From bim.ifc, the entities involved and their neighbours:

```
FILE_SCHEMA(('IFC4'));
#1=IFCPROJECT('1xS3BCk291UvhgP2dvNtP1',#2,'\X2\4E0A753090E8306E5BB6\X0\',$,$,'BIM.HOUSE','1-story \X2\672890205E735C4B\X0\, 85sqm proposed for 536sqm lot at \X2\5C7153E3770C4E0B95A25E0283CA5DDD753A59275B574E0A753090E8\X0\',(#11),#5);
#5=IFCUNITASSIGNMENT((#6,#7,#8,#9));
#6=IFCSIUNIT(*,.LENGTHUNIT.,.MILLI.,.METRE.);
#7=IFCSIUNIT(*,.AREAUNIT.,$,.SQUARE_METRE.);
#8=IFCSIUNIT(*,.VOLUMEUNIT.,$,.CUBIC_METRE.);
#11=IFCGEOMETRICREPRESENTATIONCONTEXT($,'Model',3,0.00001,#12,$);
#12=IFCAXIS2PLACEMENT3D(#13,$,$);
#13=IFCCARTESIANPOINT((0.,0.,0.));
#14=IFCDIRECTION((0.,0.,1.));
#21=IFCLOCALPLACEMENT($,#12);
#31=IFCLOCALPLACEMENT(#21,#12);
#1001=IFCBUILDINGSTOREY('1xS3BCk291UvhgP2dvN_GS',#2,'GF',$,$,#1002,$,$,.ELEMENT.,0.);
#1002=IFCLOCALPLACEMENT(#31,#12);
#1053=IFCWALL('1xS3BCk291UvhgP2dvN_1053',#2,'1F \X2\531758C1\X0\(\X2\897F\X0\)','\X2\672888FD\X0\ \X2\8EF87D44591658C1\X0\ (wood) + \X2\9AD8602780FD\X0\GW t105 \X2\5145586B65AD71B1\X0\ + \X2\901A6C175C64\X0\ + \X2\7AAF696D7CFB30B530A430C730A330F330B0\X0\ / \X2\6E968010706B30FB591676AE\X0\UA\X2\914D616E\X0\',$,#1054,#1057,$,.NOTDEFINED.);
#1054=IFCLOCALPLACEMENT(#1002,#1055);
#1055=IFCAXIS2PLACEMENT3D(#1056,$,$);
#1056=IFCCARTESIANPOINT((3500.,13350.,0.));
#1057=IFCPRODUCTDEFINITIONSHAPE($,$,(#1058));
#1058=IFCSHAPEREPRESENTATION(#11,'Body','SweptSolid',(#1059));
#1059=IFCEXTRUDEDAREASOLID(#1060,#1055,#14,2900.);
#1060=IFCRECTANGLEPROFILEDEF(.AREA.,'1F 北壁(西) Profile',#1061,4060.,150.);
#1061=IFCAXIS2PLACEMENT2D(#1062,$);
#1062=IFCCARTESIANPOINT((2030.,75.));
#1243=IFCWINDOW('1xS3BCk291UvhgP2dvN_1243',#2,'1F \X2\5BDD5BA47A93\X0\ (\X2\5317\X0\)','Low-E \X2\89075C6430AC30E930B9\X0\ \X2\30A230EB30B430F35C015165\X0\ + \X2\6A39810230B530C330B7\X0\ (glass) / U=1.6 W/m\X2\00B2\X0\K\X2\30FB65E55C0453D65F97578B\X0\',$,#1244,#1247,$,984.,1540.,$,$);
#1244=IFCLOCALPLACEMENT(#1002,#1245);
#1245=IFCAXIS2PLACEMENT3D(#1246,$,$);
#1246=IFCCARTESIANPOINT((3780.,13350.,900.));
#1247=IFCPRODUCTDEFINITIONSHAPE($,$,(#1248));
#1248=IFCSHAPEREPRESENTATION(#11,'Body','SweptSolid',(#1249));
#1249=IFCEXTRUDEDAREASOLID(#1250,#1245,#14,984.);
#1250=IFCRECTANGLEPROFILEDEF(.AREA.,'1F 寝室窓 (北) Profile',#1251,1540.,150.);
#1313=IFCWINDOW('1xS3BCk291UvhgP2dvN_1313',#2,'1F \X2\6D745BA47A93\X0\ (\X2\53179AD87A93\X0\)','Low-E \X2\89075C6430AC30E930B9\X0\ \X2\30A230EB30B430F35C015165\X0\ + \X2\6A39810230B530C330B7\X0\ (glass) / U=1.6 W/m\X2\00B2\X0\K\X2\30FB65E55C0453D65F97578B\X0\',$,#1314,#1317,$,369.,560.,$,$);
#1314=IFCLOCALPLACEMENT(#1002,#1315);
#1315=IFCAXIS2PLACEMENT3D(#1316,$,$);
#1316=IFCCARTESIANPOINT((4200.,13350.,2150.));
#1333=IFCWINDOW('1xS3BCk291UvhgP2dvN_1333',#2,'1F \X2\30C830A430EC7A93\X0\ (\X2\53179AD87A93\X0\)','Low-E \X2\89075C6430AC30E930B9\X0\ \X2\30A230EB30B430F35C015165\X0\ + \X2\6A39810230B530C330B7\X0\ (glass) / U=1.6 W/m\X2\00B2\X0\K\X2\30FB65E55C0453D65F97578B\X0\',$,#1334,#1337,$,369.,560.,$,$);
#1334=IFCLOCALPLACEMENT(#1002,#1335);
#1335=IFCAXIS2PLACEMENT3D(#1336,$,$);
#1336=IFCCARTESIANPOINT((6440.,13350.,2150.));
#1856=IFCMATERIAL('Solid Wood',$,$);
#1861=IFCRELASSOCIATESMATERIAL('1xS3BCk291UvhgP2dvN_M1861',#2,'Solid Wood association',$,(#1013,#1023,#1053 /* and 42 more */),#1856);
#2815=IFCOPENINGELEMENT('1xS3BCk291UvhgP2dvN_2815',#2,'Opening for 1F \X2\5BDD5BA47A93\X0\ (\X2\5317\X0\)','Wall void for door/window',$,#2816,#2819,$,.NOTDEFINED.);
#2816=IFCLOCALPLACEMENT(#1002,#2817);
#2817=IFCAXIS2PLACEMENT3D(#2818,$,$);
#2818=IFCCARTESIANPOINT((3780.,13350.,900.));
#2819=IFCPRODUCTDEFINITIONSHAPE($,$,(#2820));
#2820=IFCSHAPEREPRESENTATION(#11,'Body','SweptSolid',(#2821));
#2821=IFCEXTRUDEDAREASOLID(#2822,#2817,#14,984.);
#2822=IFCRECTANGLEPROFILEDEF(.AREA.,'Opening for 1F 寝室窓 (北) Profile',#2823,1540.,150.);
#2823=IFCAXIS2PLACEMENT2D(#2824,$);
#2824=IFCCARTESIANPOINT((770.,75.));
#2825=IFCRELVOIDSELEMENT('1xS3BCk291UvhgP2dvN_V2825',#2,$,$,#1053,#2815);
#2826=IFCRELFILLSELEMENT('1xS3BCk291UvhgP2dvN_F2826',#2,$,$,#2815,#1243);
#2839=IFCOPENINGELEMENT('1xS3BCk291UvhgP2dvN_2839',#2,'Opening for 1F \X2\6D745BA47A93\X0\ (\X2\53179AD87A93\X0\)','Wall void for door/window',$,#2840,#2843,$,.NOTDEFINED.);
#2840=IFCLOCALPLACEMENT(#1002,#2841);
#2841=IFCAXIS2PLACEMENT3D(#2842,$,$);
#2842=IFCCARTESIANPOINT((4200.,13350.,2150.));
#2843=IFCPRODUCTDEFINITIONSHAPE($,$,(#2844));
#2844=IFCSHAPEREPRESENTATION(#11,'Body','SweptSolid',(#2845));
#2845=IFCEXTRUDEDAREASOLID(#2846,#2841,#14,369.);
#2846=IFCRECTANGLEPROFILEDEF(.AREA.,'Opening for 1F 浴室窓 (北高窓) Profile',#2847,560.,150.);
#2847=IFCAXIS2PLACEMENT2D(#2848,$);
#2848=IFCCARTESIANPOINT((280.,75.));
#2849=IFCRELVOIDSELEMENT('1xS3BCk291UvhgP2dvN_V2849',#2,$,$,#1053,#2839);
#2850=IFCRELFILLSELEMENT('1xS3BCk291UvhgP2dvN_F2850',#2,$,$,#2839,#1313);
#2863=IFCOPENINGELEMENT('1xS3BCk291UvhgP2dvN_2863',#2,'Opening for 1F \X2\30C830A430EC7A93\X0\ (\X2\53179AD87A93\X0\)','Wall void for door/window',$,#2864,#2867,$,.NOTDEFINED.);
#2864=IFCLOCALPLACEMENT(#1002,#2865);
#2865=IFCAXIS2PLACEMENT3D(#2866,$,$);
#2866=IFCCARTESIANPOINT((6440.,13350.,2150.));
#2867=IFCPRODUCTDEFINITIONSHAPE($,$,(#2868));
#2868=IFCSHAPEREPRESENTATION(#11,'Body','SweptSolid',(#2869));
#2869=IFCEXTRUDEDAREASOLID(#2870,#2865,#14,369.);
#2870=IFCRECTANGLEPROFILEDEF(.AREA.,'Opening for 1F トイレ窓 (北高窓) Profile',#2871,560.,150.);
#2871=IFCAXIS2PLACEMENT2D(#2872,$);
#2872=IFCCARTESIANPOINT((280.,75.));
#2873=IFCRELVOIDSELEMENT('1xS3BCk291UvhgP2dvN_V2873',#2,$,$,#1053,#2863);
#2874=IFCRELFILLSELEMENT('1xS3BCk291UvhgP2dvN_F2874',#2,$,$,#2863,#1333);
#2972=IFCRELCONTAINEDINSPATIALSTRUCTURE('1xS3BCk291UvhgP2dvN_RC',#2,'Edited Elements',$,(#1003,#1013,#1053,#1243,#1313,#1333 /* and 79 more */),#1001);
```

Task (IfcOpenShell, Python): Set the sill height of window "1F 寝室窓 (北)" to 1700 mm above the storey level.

```python
import numpy as np
import ifcopenshell
import ifcopenshell.api.geometry
import ifcopenshell.geom
import ifcopenshell.util.element
import ifcopenshell.util.placement
import ifcopenshell.util.shape
import ifcopenshell.util.unit

model = ifcopenshell.open("bim.ifc")
unit_scale = ifcopenshell.util.unit.calculate_unit_scale(model)

window = model.by_guid("1xS3BCk291UvhgP2dvN_1243")
opening = window.FillsVoids[0].RelatingOpeningElement
storey = ifcopenshell.util.element.get_container(window, ifc_class="IfcBuildingStorey")
level = ifcopenshell.util.placement.get_local_placement(storey.ObjectPlacement)[2, 3]

# The opening's origin need not be at the sill, so measure its lowest point.
shape = ifcopenshell.geom.create_shape(ifcopenshell.geom.settings(), opening)
bottom = ifcopenshell.util.shape.get_shape_bottom_elevation(shape, shape.geometry) / unit_scale
dz = level + 1700.0 - bottom

shift = np.array([0.0, 0.0, dz])
# The window is not placed relative to its opening, so move both.
for product in (opening, window):
    matrix = ifcopenshell.util.placement.get_local_placement(product.ObjectPlacement)
    matrix[:3, 3] += shift
    ifcopenshell.api.geometry.edit_object_placement(model, product=product, matrix=matrix, is_si=False)

print(f"moved by {dz * unit_scale:+.3f} m")

model.write("bim_edited.ifc")
```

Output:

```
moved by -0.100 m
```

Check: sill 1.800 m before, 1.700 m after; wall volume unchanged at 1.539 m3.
